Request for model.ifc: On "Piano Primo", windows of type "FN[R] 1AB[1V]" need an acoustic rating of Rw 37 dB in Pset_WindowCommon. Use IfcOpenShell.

First a look at what the model holds.

```python
import ifcopenshell
import ifcopenshell.util.element

model = ifcopenshell.open("model.ifc")
print(model.schema)
storey = next(s for s in model.by_type("IfcBuildingStorey") if s.Name == "Piano Primo")
windows = [e for e in ifcopenshell.util.element.get_decomposition(storey) if e.is_a("IfcWindow")]
seen = {}
for e in windows:
    element_type = ifcopenshell.util.element.get_type(e)
    key = (element_type.Name if element_type != e and element_type else None, ifcopenshell.util.element.get_pset(e, "Pset_WindowCommon", "AcousticRating"))
    seen[key] = seen.get(key, 0) + 1
for (name, value), count in sorted(seen.items(), key=str):
    print(count, "x", name, "|", value)
```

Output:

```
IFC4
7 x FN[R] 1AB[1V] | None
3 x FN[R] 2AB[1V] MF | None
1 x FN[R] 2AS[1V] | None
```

```python
import ifcopenshell
import ifcopenshell.api.pset
import ifcopenshell.util.element

model = ifcopenshell.open("model.ifc")

storey = next(s for s in model.by_type("IfcBuildingStorey") if s.Name == "Piano Primo")
windows = [e for e in ifcopenshell.util.element.get_decomposition(storey) if e.is_a("IfcWindow")]

count = 0
for e in windows:
    element_type = ifcopenshell.util.element.get_type(e)
    if element_type in (None, e) or element_type.Name != "FN[R] 1AB[1V]":
        continue
    # add_pset returns the element's existing set when there is one.
    pset = ifcopenshell.api.pset.add_pset(model, product=e, name="Pset_WindowCommon")
    ifcopenshell.api.pset.edit_pset(model, pset=pset, properties={"AcousticRating": "Rw 37 dB"})
    count += 1

print(count, "windows updated")

model.write("model_v2.ifc")
```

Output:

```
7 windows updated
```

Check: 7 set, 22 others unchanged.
